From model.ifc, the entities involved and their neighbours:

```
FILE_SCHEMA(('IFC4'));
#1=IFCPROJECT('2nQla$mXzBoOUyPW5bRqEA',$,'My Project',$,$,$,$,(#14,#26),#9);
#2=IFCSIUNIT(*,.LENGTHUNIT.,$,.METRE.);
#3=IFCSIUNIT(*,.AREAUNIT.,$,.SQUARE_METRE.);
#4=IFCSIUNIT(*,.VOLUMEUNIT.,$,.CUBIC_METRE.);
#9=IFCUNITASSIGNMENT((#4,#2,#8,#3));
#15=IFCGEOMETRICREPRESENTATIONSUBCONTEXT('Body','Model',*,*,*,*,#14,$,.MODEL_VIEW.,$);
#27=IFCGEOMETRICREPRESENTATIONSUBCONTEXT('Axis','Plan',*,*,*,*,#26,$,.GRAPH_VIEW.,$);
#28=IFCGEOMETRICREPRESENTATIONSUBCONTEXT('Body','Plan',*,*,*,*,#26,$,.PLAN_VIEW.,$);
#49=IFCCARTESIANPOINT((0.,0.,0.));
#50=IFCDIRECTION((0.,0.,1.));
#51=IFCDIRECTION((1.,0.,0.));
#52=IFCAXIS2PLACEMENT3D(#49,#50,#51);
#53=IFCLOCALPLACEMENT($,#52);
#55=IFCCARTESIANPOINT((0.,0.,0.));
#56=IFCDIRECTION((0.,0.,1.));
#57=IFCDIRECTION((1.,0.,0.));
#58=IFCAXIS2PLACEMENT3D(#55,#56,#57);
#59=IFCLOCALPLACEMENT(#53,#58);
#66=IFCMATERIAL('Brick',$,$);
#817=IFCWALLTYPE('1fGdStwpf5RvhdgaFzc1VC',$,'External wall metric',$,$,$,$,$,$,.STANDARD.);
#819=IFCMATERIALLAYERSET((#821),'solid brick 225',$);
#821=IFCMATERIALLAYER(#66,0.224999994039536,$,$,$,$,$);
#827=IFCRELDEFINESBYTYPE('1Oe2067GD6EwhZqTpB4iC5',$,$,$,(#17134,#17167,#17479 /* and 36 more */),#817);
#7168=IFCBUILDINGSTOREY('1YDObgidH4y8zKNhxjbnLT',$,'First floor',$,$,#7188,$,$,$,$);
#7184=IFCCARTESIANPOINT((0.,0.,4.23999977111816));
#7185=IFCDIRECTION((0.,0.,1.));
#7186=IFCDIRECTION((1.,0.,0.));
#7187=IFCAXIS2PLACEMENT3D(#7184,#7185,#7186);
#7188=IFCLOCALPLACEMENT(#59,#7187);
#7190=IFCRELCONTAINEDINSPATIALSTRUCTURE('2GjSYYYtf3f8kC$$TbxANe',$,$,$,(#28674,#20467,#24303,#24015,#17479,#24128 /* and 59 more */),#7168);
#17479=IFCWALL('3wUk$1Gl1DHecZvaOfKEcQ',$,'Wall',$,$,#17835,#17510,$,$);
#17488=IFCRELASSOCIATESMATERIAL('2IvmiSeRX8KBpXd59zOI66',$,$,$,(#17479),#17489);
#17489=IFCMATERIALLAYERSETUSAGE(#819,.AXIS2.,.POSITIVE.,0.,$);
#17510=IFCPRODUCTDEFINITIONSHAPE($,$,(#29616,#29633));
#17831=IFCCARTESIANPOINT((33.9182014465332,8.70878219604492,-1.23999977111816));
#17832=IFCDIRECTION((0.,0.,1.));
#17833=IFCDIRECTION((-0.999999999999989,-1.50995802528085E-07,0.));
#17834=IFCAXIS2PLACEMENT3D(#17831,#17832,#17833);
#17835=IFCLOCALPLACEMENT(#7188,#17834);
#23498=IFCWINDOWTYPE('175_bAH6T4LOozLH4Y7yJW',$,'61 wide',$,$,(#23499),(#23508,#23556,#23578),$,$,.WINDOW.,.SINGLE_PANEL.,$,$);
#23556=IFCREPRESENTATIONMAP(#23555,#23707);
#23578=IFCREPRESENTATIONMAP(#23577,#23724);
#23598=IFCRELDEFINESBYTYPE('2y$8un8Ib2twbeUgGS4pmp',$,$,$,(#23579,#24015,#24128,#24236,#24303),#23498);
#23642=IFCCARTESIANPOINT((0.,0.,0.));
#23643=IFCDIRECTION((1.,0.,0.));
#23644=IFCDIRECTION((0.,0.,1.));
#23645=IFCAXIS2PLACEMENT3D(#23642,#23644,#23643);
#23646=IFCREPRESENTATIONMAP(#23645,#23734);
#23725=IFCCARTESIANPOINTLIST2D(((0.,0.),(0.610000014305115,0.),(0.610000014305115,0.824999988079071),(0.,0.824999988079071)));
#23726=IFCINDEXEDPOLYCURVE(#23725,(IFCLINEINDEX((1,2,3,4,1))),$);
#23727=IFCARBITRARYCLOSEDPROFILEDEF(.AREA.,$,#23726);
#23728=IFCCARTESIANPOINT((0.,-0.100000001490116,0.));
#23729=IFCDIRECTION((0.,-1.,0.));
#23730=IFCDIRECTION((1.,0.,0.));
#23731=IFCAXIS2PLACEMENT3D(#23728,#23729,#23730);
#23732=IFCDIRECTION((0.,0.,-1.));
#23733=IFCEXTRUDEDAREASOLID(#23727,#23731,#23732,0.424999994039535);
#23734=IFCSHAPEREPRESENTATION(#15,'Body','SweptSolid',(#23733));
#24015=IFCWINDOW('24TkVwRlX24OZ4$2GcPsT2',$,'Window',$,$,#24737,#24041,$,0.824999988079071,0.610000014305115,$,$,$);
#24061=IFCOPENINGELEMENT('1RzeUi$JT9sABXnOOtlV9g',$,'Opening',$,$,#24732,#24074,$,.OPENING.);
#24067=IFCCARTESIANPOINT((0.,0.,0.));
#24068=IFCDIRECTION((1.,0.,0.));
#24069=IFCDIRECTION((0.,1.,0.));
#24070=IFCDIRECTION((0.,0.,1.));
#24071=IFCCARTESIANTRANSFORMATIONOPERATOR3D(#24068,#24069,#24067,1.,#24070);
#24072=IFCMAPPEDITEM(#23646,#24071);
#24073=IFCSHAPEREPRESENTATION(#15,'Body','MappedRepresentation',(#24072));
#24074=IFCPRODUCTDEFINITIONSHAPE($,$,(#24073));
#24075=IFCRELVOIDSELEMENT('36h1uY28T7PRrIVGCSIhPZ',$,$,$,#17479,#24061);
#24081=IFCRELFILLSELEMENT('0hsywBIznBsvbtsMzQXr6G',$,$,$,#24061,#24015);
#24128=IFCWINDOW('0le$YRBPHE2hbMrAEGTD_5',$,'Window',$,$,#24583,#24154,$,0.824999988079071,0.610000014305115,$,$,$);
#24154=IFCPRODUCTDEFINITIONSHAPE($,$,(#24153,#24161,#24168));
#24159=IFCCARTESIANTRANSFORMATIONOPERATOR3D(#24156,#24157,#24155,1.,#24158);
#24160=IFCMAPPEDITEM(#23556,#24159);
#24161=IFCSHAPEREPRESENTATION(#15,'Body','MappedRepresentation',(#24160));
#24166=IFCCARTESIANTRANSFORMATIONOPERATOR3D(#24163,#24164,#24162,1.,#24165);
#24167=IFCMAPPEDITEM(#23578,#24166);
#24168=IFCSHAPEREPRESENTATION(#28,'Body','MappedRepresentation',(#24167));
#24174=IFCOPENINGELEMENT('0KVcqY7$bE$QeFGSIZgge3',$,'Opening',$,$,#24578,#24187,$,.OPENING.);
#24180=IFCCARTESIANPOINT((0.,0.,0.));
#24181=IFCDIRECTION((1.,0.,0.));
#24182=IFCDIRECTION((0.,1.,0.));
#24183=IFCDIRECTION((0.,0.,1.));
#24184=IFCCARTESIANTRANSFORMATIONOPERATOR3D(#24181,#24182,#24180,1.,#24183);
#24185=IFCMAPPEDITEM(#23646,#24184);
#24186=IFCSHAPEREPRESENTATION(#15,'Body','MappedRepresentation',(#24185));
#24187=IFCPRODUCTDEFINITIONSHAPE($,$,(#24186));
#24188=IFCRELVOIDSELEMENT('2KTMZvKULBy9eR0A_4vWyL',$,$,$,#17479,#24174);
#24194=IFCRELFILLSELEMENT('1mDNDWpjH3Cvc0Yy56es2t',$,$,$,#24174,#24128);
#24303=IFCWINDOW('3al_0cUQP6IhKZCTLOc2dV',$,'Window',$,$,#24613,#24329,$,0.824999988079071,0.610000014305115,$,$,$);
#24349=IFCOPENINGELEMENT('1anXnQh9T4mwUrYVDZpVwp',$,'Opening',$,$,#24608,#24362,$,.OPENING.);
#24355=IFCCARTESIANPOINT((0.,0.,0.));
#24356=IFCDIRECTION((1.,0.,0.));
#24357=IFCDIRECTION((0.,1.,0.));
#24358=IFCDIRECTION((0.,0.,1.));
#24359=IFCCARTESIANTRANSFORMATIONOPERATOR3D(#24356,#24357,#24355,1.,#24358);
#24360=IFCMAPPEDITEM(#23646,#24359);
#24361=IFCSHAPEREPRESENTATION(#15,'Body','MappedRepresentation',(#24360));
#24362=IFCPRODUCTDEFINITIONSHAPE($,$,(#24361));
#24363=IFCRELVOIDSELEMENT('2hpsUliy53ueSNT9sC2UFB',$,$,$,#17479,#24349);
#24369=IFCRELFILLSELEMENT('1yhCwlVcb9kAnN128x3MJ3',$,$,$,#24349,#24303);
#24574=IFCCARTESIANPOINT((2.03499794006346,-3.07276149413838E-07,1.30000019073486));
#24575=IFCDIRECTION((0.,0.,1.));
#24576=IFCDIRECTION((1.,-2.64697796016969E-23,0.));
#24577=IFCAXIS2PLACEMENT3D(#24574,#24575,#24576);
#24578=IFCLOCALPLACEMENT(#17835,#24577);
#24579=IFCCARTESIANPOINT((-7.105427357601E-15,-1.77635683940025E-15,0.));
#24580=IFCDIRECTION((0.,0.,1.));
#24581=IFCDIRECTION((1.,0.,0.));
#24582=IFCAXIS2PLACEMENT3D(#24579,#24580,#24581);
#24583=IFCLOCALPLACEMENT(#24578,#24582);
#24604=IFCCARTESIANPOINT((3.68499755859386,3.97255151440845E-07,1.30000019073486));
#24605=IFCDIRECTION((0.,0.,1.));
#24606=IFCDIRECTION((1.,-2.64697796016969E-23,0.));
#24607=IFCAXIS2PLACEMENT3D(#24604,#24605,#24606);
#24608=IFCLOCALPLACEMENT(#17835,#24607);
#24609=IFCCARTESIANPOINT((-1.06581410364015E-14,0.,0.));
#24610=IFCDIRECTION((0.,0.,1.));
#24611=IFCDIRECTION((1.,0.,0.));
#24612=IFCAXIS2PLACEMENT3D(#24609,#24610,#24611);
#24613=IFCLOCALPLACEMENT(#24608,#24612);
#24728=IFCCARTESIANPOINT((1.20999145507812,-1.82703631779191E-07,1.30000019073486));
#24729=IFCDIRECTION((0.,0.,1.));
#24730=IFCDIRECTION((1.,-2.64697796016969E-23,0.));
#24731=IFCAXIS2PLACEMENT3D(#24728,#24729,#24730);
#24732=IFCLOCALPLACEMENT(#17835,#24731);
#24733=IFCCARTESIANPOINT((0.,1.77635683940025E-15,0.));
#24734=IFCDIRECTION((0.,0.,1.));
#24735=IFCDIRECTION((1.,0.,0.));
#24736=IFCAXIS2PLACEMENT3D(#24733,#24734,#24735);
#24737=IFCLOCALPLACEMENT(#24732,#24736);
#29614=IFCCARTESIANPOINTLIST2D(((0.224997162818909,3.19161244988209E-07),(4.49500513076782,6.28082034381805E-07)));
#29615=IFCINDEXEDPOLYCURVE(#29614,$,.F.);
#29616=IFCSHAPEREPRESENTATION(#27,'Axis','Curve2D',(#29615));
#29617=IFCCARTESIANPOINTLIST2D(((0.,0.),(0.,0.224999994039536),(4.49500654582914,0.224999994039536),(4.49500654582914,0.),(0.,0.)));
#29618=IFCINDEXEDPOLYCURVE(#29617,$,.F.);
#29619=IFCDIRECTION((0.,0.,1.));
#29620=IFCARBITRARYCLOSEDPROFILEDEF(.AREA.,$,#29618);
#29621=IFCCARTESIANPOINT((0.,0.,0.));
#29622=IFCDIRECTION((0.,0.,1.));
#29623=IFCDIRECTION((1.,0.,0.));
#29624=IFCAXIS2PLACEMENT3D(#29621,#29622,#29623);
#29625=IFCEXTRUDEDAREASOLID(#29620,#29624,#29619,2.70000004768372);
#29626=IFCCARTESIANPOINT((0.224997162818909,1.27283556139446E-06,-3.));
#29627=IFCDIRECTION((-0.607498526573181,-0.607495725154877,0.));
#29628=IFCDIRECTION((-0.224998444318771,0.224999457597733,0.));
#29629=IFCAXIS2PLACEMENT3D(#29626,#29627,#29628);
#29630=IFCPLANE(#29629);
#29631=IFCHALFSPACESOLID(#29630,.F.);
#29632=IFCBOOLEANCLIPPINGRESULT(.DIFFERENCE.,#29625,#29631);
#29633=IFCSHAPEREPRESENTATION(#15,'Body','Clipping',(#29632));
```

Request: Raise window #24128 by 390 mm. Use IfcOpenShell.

```python
import numpy as np
import ifcopenshell
import ifcopenshell.api.geometry
import ifcopenshell.util.placement
import ifcopenshell.util.unit

model = ifcopenshell.open("model.ifc")
unit_scale = ifcopenshell.util.unit.calculate_unit_scale(model)

window = model.by_guid("0le$YRBPHE2hbMrAEGTD_5")
opening = window.FillsVoids[0].RelatingOpeningElement
dz = 0.39 / unit_scale

shift = np.array([0.0, 0.0, dz])
# The window is placed relative to its opening, so it follows when the opening moves.
matrix = ifcopenshell.util.placement.get_local_placement(opening.ObjectPlacement)
matrix[:3, 3] += shift
ifcopenshell.api.geometry.edit_object_placement(
    model, product=opening, matrix=matrix, is_si=False, should_transform_children=True
)

print(f"moved by {dz * unit_scale:+.3f} m")

model.write("model_v2.ifc")
```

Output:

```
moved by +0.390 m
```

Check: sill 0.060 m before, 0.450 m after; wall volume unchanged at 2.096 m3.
